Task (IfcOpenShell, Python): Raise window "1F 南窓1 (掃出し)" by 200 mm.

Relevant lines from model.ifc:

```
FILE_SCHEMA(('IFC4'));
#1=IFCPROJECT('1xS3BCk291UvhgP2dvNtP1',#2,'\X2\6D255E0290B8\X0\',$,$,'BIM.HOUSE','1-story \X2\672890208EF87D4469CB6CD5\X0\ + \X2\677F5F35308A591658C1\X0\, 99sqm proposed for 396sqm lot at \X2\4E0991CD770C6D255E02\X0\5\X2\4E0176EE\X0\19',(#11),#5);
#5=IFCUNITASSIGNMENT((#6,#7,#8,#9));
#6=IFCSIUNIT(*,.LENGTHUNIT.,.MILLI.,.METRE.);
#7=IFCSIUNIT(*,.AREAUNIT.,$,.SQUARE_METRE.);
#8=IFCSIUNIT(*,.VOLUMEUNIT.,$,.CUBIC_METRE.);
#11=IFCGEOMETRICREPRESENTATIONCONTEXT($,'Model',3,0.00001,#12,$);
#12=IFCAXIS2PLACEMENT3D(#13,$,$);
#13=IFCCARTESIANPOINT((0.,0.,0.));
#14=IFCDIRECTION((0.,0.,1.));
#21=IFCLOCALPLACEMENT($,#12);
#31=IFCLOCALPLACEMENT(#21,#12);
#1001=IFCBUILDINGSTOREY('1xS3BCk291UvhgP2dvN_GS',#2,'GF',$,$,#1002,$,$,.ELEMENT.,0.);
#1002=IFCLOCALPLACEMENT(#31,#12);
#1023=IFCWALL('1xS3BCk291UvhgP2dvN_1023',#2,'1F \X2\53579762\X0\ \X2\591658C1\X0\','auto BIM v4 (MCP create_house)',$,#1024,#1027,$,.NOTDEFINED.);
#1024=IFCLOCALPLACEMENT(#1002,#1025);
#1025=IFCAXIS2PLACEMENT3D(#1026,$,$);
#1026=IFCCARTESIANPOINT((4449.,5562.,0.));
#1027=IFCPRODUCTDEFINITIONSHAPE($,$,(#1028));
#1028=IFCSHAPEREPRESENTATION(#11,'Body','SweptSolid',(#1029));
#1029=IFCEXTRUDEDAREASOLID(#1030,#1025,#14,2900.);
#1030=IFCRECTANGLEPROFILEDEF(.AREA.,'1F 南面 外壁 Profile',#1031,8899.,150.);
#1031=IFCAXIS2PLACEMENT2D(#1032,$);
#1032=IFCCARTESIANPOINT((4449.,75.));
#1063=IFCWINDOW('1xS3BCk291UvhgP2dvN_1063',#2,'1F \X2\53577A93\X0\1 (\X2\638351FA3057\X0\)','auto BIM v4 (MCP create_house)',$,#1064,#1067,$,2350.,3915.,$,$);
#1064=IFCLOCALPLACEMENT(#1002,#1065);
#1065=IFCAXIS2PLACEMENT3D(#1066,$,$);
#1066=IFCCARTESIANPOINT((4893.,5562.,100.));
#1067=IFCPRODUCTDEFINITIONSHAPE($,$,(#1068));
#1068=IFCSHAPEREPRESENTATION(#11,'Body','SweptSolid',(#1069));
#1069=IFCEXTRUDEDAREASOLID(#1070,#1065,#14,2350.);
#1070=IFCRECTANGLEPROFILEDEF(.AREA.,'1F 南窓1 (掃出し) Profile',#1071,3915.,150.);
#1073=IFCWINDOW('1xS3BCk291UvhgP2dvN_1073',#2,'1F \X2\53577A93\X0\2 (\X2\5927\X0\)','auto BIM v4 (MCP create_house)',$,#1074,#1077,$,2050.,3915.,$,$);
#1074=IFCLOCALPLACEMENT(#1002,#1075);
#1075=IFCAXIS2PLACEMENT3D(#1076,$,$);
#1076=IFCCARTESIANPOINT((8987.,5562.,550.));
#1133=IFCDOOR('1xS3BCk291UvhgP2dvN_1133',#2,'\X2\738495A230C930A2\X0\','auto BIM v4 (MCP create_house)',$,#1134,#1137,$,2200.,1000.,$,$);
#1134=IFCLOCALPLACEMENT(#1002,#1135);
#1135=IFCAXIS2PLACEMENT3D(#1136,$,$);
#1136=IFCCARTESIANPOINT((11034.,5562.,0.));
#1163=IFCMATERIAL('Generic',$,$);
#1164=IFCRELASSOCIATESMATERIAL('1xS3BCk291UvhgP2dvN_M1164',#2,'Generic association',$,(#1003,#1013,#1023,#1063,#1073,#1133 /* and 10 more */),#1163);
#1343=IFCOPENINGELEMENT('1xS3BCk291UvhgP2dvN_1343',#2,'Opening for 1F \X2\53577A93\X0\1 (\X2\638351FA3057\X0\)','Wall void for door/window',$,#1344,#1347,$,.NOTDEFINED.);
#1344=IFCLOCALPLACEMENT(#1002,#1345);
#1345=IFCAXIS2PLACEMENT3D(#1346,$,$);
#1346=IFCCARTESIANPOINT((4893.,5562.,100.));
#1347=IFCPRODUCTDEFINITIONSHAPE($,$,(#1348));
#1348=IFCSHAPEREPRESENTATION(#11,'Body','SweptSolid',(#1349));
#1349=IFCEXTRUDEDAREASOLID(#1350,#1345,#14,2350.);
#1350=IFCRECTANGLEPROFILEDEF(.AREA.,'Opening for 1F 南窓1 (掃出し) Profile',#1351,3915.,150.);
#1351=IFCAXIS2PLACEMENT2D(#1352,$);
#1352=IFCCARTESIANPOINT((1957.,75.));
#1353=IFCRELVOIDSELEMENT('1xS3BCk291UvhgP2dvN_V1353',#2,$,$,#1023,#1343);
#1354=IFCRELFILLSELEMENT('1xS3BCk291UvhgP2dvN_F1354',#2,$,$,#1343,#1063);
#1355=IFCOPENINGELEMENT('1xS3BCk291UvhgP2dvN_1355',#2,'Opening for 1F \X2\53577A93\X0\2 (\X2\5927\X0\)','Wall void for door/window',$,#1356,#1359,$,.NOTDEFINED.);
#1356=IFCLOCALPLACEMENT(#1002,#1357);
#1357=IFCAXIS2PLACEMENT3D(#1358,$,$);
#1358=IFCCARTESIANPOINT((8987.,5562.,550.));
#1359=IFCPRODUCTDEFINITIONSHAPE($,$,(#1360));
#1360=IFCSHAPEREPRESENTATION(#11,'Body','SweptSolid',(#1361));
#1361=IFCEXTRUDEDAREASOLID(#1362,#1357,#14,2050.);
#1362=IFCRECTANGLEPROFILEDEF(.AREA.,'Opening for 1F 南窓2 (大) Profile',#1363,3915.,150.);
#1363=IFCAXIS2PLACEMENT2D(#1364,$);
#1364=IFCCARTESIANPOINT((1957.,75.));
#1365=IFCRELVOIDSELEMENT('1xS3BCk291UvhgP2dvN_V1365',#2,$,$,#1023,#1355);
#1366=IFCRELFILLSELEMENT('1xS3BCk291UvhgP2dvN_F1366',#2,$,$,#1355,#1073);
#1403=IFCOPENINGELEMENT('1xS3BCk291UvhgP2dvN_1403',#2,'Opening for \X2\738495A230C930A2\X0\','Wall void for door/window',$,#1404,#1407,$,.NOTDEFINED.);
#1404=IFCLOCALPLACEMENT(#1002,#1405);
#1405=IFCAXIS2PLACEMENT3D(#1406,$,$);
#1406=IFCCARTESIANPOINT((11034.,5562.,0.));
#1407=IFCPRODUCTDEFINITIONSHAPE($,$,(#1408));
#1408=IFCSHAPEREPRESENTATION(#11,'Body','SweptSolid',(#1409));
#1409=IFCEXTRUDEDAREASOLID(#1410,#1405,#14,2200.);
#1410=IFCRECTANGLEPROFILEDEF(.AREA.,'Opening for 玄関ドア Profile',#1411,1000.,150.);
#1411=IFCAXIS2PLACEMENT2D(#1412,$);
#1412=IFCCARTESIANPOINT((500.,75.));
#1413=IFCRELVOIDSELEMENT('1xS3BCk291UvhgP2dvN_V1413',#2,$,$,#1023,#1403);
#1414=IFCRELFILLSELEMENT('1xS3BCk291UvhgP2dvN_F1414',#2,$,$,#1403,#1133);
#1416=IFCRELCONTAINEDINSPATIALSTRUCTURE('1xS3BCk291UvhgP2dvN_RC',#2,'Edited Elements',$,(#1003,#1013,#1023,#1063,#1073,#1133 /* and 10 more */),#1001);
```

```python
import numpy as np
import ifcopenshell
import ifcopenshell.api.geometry
import ifcopenshell.util.placement
import ifcopenshell.util.unit

model = ifcopenshell.open("model.ifc")
unit_scale = ifcopenshell.util.unit.calculate_unit_scale(model)

window = model.by_guid("1xS3BCk291UvhgP2dvN_1063")
opening = window.FillsVoids[0].RelatingOpeningElement
dz = 200.0

shift = np.array([0.0, 0.0, dz])
# The window is not placed relative to its opening, so move both.
for product in (opening, window):
    matrix = ifcopenshell.util.placement.get_local_placement(product.ObjectPlacement)
    matrix[:3, 3] += shift
    ifcopenshell.api.geometry.edit_object_placement(model, product=product, matrix=matrix, is_si=False)

print(f"moved by {dz * unit_scale:+.3f} m")

model.write("model_updated.ifc")
```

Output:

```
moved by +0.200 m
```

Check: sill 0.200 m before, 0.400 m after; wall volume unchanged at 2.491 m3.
